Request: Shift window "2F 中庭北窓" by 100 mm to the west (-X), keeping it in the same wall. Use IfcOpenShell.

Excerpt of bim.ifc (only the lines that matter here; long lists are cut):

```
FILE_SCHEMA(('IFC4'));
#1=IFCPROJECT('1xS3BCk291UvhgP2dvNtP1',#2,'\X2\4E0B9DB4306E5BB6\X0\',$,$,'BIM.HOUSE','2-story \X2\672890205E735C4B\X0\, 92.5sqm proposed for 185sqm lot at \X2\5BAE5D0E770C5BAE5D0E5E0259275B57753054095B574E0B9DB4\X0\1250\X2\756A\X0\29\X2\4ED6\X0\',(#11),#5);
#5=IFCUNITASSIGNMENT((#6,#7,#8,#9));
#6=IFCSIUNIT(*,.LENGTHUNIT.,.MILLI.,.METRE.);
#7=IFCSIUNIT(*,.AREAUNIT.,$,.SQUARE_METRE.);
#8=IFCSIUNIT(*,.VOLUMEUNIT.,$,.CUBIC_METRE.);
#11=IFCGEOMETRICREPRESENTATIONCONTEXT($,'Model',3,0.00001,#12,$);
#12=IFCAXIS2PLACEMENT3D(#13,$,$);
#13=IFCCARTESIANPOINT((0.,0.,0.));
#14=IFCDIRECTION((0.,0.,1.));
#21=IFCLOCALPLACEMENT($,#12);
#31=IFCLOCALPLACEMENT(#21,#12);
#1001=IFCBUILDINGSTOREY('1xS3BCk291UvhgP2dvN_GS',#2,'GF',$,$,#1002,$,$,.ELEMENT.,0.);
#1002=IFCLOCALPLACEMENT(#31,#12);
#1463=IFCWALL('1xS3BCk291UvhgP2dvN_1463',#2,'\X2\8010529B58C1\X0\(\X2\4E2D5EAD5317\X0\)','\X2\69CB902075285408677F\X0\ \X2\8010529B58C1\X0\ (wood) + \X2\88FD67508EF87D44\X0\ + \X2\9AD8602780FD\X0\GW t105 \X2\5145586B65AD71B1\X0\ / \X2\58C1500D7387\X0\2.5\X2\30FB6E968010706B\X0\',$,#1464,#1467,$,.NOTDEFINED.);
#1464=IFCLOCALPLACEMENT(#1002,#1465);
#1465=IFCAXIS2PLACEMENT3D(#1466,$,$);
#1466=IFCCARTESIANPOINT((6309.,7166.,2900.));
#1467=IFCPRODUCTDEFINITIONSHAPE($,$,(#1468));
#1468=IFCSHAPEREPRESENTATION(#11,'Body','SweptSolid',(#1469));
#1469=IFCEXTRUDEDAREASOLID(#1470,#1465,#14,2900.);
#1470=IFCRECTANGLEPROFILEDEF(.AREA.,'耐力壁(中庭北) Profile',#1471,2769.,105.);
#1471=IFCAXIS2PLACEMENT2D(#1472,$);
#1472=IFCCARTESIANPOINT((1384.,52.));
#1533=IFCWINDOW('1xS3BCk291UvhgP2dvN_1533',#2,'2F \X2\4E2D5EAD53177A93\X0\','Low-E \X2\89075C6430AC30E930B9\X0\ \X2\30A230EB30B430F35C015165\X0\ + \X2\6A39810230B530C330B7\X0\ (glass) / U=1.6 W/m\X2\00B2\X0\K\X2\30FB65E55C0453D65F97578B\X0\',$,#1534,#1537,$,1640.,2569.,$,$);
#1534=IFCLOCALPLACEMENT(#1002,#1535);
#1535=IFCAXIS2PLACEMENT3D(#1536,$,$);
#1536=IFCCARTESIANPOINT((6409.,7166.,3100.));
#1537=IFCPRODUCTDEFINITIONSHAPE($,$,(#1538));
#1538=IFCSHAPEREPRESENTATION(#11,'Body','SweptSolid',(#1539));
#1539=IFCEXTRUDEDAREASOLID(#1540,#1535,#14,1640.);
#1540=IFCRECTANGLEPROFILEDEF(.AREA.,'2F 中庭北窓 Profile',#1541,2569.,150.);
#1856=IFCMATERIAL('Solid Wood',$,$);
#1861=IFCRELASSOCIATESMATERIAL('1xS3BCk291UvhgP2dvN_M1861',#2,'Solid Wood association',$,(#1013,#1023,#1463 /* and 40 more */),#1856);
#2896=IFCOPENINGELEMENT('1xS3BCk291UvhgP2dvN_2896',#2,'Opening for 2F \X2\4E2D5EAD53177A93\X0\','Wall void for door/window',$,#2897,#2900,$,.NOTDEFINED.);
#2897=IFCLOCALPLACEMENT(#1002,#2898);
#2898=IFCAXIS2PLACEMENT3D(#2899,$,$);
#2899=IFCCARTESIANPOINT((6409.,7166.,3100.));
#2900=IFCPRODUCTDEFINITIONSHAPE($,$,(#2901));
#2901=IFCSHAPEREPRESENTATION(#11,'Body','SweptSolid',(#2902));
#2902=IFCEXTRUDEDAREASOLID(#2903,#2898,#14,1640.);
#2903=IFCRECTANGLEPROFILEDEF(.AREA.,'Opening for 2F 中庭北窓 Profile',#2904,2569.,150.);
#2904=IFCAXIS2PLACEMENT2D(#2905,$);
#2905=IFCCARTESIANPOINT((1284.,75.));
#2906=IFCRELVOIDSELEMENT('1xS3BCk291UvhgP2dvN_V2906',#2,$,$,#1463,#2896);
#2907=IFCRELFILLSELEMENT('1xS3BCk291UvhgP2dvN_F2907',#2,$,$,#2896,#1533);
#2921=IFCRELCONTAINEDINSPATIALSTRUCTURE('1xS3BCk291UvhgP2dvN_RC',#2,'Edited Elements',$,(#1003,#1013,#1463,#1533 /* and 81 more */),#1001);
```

```python
import ifcopenshell
import ifcopenshell.api.geometry
import ifcopenshell.util.placement

model = ifcopenshell.open("bim.ifc")

window = model.by_guid("1xS3BCk291UvhgP2dvN_1533")
opening = window.FillsVoids[0].RelatingOpeningElement
wall = opening.VoidsElements[0].RelatingBuildingElement

wall_matrix = ifcopenshell.util.placement.get_local_placement(wall.ObjectPlacement)
shift = wall_matrix[:3, 0] * -100.0
before = ifcopenshell.util.placement.get_local_placement(window.ObjectPlacement)[:3, 3].copy()

# The window is not placed relative to its opening, so move both.
for product in (opening, window):
    matrix = ifcopenshell.util.placement.get_local_placement(product.ObjectPlacement)
    matrix[:3, 3] += shift
    ifcopenshell.api.geometry.edit_object_placement(model, product=product, matrix=matrix, is_si=False)

after = ifcopenshell.util.placement.get_local_placement(window.ObjectPlacement)[:3, 3]
print("window moved by", (after - before).round(3) + 0.0)

model.write("bim_updated.ifc")
```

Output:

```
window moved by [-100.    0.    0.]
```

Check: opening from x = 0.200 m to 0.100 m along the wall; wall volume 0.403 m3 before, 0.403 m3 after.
